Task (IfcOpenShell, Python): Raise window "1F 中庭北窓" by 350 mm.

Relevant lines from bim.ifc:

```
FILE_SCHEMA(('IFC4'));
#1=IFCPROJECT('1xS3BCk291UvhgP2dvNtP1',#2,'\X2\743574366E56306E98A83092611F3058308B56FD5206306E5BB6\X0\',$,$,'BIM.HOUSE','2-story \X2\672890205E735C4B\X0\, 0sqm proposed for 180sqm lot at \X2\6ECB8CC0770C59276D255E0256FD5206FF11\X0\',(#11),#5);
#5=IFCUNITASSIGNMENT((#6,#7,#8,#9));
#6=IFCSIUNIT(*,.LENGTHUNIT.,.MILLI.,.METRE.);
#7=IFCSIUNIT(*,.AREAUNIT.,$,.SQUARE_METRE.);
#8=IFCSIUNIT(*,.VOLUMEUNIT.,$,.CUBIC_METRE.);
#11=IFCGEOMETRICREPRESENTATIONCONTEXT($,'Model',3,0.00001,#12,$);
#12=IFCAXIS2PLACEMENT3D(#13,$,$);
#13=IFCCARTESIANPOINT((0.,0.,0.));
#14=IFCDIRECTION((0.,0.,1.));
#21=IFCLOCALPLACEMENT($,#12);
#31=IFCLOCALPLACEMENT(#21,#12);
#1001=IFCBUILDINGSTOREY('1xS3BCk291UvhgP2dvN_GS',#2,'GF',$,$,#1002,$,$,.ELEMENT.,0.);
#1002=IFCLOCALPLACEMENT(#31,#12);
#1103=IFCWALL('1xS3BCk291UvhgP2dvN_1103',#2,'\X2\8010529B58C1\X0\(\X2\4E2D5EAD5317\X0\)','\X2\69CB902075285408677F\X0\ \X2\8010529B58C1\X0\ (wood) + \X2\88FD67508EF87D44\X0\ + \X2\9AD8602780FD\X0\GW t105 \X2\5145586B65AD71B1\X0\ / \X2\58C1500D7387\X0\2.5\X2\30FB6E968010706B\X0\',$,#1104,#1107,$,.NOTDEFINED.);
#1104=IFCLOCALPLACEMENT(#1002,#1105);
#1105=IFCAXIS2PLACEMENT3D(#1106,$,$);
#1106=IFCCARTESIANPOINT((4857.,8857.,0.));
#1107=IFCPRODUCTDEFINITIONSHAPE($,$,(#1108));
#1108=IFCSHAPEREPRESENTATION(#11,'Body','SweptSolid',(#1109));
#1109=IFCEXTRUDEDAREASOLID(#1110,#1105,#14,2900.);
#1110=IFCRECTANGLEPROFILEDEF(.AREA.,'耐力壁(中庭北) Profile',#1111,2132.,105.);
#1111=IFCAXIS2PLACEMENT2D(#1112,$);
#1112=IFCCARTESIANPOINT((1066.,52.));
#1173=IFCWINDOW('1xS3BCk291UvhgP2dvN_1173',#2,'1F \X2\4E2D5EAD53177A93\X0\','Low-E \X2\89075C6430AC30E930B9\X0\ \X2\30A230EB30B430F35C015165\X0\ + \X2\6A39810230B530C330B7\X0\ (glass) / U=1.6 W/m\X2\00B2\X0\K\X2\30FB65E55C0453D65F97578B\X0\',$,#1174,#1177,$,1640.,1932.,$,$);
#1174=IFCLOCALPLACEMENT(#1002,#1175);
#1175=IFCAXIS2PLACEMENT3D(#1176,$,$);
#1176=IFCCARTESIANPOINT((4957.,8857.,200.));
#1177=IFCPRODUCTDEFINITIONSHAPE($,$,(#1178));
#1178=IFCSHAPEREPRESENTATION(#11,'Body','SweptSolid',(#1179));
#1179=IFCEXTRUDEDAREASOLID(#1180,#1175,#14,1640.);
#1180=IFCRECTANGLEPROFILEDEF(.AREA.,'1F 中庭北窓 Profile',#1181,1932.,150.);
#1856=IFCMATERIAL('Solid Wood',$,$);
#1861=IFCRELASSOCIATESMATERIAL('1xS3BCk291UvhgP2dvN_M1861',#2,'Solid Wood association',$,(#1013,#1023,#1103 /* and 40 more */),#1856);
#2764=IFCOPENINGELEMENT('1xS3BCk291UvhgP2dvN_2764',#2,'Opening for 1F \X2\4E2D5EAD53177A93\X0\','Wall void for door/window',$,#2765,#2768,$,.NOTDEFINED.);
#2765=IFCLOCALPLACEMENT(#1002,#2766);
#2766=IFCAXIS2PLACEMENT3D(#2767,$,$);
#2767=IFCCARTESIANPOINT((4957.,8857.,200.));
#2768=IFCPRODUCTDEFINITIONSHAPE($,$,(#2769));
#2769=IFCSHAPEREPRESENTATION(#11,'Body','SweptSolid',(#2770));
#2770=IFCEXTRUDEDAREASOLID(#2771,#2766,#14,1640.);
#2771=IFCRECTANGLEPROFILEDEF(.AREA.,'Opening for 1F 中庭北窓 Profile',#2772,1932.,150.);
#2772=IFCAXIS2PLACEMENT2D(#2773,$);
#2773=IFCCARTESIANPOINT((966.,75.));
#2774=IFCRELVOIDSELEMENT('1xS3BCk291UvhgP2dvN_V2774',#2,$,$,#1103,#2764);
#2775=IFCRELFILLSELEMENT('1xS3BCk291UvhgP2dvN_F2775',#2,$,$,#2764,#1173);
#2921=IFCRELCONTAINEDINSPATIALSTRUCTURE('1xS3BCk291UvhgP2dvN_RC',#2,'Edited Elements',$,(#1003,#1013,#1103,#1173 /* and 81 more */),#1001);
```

```python
import numpy as np
import ifcopenshell
import ifcopenshell.api.geometry
import ifcopenshell.util.placement
import ifcopenshell.util.unit

model = ifcopenshell.open("bim.ifc")
unit_scale = ifcopenshell.util.unit.calculate_unit_scale(model)

window = model.by_guid("1xS3BCk291UvhgP2dvN_1173")
opening = window.FillsVoids[0].RelatingOpeningElement
dz = 0.35 / unit_scale

shift = np.array([0.0, 0.0, dz])
# The window is not placed relative to its opening, so move both.
for product in (opening, window):
    matrix = ifcopenshell.util.placement.get_local_placement(product.ObjectPlacement)
    matrix[:3, 3] += shift
    ifcopenshell.api.geometry.edit_object_placement(model, product=product, matrix=matrix, is_si=False)

print(f"moved by {dz * unit_scale:+.3f} m")

model.write("bim_edited.ifc")
```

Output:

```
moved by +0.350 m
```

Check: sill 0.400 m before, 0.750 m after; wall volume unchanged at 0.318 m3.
